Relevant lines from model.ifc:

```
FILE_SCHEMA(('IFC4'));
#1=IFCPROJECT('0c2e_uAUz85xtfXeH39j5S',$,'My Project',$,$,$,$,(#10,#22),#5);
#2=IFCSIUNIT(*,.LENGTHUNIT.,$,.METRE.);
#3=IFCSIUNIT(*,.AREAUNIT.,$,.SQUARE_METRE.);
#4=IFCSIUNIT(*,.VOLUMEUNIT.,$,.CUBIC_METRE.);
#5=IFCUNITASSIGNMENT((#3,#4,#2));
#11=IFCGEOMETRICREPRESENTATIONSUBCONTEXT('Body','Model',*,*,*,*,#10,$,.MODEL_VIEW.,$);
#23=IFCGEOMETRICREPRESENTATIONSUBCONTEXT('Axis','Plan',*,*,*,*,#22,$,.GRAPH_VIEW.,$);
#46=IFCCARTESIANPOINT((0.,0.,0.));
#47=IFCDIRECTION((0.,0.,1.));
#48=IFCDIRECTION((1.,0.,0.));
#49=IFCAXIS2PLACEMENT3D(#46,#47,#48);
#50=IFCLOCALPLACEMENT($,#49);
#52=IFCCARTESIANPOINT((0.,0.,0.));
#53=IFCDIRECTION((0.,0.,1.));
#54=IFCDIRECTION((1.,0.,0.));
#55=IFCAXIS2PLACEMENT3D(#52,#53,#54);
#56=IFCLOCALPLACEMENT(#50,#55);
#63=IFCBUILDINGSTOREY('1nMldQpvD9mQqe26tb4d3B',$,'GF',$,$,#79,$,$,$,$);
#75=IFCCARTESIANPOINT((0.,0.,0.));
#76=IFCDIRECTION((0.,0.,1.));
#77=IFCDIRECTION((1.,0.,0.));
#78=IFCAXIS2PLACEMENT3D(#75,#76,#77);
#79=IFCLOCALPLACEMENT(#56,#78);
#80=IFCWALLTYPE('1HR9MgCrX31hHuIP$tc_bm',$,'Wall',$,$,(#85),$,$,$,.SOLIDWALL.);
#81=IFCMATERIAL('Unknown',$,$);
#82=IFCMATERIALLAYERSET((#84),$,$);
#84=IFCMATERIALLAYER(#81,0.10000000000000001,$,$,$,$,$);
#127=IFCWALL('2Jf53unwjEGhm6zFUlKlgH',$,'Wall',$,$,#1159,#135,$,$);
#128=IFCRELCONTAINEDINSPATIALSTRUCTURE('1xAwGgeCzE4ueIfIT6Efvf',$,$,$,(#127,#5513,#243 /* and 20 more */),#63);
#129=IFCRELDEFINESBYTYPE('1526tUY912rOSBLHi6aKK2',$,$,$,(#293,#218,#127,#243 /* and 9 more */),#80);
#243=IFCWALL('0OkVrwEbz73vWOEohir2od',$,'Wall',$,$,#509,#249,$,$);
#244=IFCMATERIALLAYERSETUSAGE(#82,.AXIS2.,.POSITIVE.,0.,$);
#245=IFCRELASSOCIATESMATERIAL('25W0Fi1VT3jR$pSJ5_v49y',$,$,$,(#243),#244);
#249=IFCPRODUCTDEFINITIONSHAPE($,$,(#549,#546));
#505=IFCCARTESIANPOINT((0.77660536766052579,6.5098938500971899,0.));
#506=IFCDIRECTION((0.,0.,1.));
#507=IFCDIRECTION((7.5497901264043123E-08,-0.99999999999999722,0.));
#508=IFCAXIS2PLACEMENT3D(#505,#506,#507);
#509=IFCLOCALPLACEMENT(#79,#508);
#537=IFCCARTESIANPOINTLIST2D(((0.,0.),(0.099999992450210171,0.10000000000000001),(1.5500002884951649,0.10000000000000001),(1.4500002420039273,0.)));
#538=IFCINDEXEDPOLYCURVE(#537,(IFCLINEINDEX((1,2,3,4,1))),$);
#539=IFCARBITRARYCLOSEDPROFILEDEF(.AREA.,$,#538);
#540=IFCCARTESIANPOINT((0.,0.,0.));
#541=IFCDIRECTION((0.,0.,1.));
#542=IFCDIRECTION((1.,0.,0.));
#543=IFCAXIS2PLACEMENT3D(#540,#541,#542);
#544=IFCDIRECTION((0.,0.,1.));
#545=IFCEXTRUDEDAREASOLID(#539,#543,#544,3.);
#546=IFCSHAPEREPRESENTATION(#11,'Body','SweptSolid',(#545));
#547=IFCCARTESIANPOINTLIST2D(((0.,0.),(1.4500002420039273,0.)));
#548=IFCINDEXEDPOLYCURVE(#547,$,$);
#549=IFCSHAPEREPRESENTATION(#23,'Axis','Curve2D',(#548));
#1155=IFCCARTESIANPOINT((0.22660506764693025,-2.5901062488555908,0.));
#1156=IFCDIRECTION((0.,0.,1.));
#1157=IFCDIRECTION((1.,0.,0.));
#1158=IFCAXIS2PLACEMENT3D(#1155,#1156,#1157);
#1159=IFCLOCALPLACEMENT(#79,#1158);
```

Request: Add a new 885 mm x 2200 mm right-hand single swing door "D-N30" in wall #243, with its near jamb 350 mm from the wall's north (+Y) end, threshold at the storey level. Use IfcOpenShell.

```python
import numpy as np
import ifcopenshell
import ifcopenshell.api.feature
import ifcopenshell.api.geometry
import ifcopenshell.api.root
import ifcopenshell.api.spatial
import ifcopenshell.geom
import ifcopenshell.util.element
import ifcopenshell.util.placement
import ifcopenshell.util.representation
import ifcopenshell.util.shape
import ifcopenshell.util.unit

model = ifcopenshell.open("model.ifc")
unit_scale = ifcopenshell.util.unit.calculate_unit_scale(model)
settings = ifcopenshell.geom.settings()


def volume(element):
    """Net volume in cubic metres, openings subtracted."""
    shape = ifcopenshell.geom.create_shape(settings, element)
    return ifcopenshell.util.shape.get_volume(shape.geometry)


wall = model.by_guid("0OkVrwEbz73vWOEohir2od")
storey = ifcopenshell.util.element.get_container(wall, ifc_class="IfcBuildingStorey")
context = ifcopenshell.util.representation.get_context(model, "Model", "Body", "MODEL_VIEW")
before = volume(wall)

width, height, from_end, sill = 0.885, 2.2, 0.35, 0.0  # metres

# The wall runs along its own X axis, and the end named is its -X end.
wall_shape = ifcopenshell.geom.create_shape(settings, wall)
x, y, z = ifcopenshell.util.shape.get_vertices(wall_shape.geometry).T
start = x.min() + from_end
face, thickness = float(y.min()), float(y.max() - y.min())
wall_matrix = ifcopenshell.util.placement.get_local_placement(wall.ObjectPlacement)
level = ifcopenshell.util.placement.get_local_placement(storey.ObjectPlacement)[2, 3]


def in_wall(x, y):
    """Placement at x, y metres in the wall's axes, at sill height."""
    matrix = wall_matrix.copy()
    matrix[:, 3] = wall_matrix @ np.array([x / unit_scale, y / unit_scale, 0.0, 1.0])
    matrix[2, 3] = level + sill / unit_scale
    return matrix


# Opening: a box that overshoots both wall faces by 50 mm.
opening = ifcopenshell.api.root.create_entity(model, ifc_class="IfcOpeningElement", predefined_type="OPENING")
box = ifcopenshell.api.geometry.add_wall_representation(
    model, context=context, length=width, height=height, thickness=thickness + 0.1
)
ifcopenshell.api.geometry.assign_representation(model, product=opening, representation=box)
ifcopenshell.api.geometry.edit_object_placement(model, product=opening, matrix=in_wall(start, face - 0.05), is_si=False)
ifcopenshell.api.feature.add_feature(model, feature=opening, element=wall)

door = ifcopenshell.api.root.create_entity(model, ifc_class="IfcDoor", name="D-N30", predefined_type="DOOR")
door.OverallWidth, door.OverallHeight = width / unit_scale, height / unit_scale
door.OperationType = "SINGLE_SWING_RIGHT"
body = ifcopenshell.api.geometry.add_door_representation(
    model,
    context=context,
    overall_width=door.OverallWidth,
    overall_height=door.OverallHeight,
    operation_type="SINGLE_SWING_RIGHT",
    lining_properties={"LiningDepth": thickness / unit_scale, "ThresholdDepth": thickness / unit_scale},
)
ifcopenshell.api.geometry.assign_representation(model, product=door, representation=body)
ifcopenshell.api.spatial.assign_container(model, products=[door], relating_structure=storey)
ifcopenshell.api.feature.add_filling(model, opening=opening, element=door)

# The lining spans the wall, so the door starts at the wall face.
ifcopenshell.api.geometry.edit_object_placement(model, product=door, matrix=in_wall(start, face), is_si=False)

after = volume(wall)

print(f"wall volume {before:.3f} -> {after:.3f} m3")

model.write("model-out.ifc")
```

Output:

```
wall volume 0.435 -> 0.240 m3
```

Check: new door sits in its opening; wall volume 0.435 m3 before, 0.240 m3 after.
